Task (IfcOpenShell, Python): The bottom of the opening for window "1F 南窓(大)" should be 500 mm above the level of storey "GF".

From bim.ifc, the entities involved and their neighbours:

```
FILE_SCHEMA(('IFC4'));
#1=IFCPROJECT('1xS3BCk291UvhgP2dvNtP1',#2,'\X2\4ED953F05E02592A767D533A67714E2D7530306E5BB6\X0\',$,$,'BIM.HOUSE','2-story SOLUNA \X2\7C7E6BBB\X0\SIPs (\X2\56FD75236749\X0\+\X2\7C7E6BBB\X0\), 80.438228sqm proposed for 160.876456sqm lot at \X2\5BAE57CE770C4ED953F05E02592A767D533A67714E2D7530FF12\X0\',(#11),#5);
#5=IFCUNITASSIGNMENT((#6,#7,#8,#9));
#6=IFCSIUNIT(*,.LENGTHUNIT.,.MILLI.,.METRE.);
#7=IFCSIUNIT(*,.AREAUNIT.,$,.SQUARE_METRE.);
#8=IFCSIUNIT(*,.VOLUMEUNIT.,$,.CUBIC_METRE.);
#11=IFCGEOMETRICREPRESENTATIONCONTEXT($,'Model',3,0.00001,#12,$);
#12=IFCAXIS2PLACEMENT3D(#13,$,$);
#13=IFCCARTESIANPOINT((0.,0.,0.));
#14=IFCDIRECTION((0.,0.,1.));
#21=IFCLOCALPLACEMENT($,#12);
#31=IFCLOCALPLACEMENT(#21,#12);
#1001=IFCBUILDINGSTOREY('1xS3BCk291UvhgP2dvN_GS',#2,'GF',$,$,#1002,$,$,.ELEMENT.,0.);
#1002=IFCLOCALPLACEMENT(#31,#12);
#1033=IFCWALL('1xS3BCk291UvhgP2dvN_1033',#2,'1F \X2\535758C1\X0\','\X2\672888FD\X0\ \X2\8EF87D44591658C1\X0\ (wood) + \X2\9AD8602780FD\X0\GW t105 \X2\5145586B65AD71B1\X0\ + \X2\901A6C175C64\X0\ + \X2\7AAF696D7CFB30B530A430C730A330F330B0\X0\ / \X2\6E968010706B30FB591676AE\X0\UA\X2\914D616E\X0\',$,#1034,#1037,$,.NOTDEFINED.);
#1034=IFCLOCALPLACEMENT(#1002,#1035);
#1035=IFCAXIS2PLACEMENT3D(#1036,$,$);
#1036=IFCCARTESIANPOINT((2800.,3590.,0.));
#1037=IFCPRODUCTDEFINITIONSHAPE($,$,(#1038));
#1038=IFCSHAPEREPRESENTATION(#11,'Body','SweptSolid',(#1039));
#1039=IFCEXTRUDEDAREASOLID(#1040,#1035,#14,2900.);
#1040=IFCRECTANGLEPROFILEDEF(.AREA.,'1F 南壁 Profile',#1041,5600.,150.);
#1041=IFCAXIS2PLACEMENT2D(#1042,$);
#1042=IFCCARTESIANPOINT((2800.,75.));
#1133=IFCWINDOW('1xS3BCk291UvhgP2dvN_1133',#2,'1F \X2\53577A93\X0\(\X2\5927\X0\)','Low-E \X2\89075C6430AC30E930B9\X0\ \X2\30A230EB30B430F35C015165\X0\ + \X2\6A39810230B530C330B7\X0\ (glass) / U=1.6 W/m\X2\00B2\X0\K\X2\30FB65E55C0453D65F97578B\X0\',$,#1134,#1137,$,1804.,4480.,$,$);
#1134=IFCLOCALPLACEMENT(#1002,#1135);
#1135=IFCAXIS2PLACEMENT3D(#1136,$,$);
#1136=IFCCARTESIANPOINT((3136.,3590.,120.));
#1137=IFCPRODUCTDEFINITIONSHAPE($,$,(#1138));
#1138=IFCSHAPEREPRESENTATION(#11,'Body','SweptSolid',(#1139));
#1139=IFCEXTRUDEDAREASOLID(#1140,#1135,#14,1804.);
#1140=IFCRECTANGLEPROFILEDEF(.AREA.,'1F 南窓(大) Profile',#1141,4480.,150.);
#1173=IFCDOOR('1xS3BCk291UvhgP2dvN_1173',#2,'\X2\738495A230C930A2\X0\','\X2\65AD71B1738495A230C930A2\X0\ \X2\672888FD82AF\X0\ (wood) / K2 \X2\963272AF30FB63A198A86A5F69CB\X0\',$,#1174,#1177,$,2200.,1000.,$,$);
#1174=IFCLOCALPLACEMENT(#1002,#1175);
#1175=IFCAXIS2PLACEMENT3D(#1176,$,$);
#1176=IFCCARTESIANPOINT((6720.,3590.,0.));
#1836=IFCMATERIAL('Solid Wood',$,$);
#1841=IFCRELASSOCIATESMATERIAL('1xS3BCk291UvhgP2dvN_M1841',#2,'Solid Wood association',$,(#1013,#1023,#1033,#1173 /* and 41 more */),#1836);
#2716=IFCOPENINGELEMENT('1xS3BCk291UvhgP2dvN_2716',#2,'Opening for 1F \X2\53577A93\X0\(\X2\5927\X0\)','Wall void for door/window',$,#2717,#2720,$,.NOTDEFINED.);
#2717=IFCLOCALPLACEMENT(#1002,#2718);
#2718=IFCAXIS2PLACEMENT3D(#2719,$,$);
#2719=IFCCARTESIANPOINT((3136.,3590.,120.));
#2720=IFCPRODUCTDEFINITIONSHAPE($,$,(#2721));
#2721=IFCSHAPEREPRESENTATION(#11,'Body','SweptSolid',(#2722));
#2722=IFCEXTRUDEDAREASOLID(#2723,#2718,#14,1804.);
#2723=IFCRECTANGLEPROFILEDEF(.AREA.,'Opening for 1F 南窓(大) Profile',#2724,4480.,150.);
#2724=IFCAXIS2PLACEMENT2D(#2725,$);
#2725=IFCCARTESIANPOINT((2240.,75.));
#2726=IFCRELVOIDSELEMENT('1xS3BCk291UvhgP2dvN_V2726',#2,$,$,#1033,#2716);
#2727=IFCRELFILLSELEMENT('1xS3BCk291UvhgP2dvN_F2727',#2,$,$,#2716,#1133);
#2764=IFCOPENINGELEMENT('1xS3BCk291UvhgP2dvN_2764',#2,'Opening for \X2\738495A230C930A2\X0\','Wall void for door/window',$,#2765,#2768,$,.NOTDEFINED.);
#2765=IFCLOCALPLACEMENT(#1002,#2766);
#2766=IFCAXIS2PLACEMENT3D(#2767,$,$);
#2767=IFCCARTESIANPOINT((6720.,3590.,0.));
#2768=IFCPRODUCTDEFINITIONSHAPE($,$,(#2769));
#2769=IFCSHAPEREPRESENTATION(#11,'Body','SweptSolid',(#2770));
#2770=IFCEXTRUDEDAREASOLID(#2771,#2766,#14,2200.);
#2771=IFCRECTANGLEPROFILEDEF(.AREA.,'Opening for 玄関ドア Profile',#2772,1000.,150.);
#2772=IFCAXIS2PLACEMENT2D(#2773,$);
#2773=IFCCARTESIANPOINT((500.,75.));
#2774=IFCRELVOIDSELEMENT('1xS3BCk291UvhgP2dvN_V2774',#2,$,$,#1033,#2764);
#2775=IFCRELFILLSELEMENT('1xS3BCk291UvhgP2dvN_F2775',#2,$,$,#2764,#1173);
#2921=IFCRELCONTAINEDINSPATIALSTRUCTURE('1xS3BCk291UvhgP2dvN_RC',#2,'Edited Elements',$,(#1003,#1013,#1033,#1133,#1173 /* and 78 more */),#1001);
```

```python
import numpy as np
import ifcopenshell
import ifcopenshell.api.geometry
import ifcopenshell.geom
import ifcopenshell.util.element
import ifcopenshell.util.placement
import ifcopenshell.util.shape
import ifcopenshell.util.unit

model = ifcopenshell.open("bim.ifc")
unit_scale = ifcopenshell.util.unit.calculate_unit_scale(model)

window = model.by_id(1133)
opening = window.FillsVoids[0].RelatingOpeningElement
storey = ifcopenshell.util.element.get_container(window, ifc_class="IfcBuildingStorey")
level = ifcopenshell.util.placement.get_local_placement(storey.ObjectPlacement)[2, 3]

# The opening's origin need not be at the sill, so measure its lowest point.
shape = ifcopenshell.geom.create_shape(ifcopenshell.geom.settings(), opening)
bottom = ifcopenshell.util.shape.get_shape_bottom_elevation(shape, shape.geometry) / unit_scale
dz = level + 0.5 / unit_scale - bottom

shift = np.array([0.0, 0.0, dz])
# The window is not placed relative to its opening, so move both.
for product in (opening, window):
    matrix = ifcopenshell.util.placement.get_local_placement(product.ObjectPlacement)
    matrix[:3, 3] += shift
    ifcopenshell.api.geometry.edit_object_placement(model, product=product, matrix=matrix, is_si=False)

print(f"moved by {dz * unit_scale:+.3f} m")

model.write("bim-out.ifc")
```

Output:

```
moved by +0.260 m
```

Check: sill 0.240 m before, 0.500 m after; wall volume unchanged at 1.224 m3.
